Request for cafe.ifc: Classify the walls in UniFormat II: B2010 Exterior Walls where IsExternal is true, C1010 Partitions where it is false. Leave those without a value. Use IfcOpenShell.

First a look at what the model holds.

```python
import ifcopenshell
import ifcopenshell.util.element

model = ifcopenshell.open("cafe.ifc")
print(model.schema)
print("classifications:", [c.Name for c in model.by_type("IfcClassification")])
values = [ifcopenshell.util.element.get_pset(e, "Pset_WallCommon", "IsExternal") for e in model.by_type("IfcWall")]
for value in (True, False, None):
    print("IsExternal", value, values.count(value))
```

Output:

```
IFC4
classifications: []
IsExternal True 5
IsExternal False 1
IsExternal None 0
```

```python
import ifcopenshell
import ifcopenshell.api.classification
import ifcopenshell.util.element

model = ifcopenshell.open("cafe.ifc")

system = ifcopenshell.api.classification.add_classification(model, classification="UniFormat II")

walls = model.by_type("IfcWall")
external = {e: ifcopenshell.util.element.get_pset(e, "Pset_WallCommon", "IsExternal") for e in walls}
for flag, code, name in ((True, "B2010", "Exterior Walls"), (False, "C1010", "Partitions")):
    products = [e for e in walls if external[e] is flag]
    ifcopenshell.api.classification.add_reference(
        model, products=products, classification=system, identification=code, name=name
    )
    print(code, len(products))

model.write("cafe-out.ifc")
```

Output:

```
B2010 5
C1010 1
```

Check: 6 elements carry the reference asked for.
